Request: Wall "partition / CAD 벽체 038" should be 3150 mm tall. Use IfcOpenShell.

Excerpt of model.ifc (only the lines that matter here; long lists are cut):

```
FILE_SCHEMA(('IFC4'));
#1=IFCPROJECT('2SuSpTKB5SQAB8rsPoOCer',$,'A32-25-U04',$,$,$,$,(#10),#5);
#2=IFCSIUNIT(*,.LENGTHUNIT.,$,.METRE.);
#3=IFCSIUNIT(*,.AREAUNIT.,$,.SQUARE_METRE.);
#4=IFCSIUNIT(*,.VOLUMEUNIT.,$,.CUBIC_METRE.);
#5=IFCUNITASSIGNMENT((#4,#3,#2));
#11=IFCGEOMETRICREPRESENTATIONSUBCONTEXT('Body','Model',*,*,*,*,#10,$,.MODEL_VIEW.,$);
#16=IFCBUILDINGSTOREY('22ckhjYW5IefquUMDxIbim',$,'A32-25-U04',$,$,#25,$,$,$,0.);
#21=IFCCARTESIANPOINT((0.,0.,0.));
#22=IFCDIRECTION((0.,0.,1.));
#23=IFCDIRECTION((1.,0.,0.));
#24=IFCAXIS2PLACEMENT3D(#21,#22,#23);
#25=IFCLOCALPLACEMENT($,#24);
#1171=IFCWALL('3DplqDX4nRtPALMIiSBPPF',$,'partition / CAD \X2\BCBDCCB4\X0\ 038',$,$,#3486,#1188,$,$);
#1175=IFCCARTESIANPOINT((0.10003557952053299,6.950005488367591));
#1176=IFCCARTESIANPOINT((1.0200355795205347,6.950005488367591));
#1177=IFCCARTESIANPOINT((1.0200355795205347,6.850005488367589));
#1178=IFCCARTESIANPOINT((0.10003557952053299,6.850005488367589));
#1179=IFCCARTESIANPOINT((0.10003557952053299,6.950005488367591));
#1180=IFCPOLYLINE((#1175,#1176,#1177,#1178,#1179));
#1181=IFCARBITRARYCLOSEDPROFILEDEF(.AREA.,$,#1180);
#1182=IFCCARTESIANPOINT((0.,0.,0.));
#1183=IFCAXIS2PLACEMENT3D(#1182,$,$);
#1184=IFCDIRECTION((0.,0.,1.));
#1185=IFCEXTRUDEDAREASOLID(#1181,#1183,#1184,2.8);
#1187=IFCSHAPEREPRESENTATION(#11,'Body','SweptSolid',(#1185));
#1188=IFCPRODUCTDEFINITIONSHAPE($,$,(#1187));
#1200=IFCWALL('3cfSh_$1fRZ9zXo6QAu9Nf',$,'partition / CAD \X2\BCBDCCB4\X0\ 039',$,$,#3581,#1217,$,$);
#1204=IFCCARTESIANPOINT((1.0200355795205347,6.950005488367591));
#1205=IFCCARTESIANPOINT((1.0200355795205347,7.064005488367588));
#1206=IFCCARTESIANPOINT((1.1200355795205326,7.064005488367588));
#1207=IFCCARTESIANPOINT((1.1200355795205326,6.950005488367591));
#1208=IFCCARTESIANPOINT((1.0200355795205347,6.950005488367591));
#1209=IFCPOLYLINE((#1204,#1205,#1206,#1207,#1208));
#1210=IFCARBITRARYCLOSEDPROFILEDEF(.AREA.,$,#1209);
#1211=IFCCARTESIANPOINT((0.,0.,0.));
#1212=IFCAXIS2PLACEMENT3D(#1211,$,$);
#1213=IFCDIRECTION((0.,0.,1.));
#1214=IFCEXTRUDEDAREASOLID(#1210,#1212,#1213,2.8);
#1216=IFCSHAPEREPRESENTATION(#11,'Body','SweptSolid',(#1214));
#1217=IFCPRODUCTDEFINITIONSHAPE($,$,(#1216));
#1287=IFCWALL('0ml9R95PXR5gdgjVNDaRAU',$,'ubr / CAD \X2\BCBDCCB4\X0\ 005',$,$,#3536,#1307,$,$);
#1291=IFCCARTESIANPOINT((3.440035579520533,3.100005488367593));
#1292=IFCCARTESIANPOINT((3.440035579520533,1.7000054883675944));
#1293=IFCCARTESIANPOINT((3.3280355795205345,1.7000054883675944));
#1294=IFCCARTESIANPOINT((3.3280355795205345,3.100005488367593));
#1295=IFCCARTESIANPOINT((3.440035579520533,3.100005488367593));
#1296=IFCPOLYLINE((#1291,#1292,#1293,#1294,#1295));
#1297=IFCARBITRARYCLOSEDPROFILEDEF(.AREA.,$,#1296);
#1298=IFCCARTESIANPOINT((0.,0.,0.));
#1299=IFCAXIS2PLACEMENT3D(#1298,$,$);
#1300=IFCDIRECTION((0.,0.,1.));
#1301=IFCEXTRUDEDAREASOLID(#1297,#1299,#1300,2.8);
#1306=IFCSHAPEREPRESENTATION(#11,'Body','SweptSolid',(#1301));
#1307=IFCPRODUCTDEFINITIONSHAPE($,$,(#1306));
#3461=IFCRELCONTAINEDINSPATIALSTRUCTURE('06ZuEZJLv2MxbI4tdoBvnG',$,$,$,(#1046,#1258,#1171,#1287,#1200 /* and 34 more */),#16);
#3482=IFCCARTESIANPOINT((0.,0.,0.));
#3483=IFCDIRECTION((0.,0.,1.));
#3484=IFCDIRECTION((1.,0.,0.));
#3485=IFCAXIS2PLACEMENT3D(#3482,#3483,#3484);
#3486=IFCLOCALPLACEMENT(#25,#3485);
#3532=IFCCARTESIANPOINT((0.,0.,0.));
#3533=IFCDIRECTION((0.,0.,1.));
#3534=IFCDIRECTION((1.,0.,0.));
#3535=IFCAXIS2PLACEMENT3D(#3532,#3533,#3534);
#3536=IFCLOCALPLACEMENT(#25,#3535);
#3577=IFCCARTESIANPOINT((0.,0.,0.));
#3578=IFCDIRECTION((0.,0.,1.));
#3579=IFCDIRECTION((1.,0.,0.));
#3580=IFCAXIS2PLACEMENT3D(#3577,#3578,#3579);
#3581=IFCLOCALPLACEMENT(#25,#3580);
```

```python
import ifcopenshell
import ifcopenshell.geom
import ifcopenshell.util.representation
import ifcopenshell.util.shape

model = ifcopenshell.open("model.ifc")
settings = ifcopenshell.geom.settings()


def volume(element):
    """Net volume in cubic metres, openings subtracted."""
    shape = ifcopenshell.geom.create_shape(settings, element)
    return ifcopenshell.util.shape.get_volume(shape.geometry)


wall = model.by_guid("3DplqDX4nRtPALMIiSBPPF")
before = volume(wall)

body = ifcopenshell.util.representation.get_representation(wall, "Model", "Body")
solid = body.Items[0]
old_height = solid.Depth
solid.Depth = 3.15
after = volume(wall)

print(f"height {old_height:g} -> {solid.Depth:g}, volume {before:.3f} -> {after:.3f} m3")

model.write("model_updated.ifc")
```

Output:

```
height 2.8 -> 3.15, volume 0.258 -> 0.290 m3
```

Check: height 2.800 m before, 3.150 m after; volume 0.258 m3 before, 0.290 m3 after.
